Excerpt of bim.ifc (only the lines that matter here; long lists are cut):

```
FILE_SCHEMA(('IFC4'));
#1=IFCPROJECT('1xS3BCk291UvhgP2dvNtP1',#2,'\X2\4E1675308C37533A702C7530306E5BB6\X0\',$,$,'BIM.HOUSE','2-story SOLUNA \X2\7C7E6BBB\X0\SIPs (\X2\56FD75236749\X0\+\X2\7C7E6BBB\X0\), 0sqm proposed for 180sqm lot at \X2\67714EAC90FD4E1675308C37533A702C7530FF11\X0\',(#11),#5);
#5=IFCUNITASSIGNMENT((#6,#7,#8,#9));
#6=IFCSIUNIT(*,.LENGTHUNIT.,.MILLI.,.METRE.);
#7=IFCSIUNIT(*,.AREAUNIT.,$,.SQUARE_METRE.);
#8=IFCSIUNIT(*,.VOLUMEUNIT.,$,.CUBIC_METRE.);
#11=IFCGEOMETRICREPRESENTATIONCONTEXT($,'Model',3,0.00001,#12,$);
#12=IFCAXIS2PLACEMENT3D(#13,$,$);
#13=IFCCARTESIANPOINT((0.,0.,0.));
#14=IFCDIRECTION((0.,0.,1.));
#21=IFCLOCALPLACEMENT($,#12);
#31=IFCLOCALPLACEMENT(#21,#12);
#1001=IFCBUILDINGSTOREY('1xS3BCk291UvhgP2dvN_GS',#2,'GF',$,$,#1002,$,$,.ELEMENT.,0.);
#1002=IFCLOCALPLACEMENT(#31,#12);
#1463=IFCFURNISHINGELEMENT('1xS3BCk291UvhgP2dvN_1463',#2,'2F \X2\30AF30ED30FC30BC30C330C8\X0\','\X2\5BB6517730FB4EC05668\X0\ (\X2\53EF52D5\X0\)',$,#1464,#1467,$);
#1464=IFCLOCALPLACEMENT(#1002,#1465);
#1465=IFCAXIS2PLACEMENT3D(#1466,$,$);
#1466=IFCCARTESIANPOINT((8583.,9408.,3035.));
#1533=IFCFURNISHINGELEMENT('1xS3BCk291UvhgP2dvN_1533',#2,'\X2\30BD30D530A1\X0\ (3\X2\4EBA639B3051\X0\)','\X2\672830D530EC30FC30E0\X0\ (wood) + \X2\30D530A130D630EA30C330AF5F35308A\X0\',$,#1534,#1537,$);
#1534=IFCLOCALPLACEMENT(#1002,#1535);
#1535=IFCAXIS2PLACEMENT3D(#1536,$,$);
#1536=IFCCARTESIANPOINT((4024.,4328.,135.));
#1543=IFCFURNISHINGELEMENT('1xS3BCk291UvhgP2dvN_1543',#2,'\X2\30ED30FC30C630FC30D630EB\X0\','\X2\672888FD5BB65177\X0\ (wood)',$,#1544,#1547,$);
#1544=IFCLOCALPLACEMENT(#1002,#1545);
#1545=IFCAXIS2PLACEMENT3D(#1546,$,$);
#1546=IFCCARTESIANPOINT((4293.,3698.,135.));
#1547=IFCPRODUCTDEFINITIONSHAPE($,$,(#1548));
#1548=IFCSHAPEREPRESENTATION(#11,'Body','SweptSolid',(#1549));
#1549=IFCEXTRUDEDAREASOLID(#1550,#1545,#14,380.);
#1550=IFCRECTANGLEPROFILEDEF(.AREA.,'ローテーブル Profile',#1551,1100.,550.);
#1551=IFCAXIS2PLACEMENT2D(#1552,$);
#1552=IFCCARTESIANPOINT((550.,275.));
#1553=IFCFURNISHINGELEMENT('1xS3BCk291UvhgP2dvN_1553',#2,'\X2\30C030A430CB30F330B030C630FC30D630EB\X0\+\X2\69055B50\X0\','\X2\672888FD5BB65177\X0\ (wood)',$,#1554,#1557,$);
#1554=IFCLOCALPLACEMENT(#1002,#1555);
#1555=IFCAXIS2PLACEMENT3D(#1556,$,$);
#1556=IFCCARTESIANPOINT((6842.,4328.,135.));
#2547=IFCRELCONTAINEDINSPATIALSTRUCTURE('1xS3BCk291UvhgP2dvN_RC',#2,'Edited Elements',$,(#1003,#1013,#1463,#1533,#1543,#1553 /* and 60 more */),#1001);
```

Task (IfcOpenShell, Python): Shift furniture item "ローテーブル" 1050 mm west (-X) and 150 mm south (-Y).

```python
import ifcopenshell
import ifcopenshell.api.geometry
import ifcopenshell.util.placement

model = ifcopenshell.open("bim.ifc")

item = model.by_guid("1xS3BCk291UvhgP2dvN_1543")
matrix = ifcopenshell.util.placement.get_local_placement(item.ObjectPlacement)
matrix[0, 3] -= 1050.0
matrix[1, 3] -= 150.0
ifcopenshell.api.geometry.edit_object_placement(model, product=item, matrix=matrix, is_si=False)

print(ifcopenshell.util.placement.get_local_placement(item.ObjectPlacement).round(3) + 0.0)

model.write("bim_rev.ifc")
```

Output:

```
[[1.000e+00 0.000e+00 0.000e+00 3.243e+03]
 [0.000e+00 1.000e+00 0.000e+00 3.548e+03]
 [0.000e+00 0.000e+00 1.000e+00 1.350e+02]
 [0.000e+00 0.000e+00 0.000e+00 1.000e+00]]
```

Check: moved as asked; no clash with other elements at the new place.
